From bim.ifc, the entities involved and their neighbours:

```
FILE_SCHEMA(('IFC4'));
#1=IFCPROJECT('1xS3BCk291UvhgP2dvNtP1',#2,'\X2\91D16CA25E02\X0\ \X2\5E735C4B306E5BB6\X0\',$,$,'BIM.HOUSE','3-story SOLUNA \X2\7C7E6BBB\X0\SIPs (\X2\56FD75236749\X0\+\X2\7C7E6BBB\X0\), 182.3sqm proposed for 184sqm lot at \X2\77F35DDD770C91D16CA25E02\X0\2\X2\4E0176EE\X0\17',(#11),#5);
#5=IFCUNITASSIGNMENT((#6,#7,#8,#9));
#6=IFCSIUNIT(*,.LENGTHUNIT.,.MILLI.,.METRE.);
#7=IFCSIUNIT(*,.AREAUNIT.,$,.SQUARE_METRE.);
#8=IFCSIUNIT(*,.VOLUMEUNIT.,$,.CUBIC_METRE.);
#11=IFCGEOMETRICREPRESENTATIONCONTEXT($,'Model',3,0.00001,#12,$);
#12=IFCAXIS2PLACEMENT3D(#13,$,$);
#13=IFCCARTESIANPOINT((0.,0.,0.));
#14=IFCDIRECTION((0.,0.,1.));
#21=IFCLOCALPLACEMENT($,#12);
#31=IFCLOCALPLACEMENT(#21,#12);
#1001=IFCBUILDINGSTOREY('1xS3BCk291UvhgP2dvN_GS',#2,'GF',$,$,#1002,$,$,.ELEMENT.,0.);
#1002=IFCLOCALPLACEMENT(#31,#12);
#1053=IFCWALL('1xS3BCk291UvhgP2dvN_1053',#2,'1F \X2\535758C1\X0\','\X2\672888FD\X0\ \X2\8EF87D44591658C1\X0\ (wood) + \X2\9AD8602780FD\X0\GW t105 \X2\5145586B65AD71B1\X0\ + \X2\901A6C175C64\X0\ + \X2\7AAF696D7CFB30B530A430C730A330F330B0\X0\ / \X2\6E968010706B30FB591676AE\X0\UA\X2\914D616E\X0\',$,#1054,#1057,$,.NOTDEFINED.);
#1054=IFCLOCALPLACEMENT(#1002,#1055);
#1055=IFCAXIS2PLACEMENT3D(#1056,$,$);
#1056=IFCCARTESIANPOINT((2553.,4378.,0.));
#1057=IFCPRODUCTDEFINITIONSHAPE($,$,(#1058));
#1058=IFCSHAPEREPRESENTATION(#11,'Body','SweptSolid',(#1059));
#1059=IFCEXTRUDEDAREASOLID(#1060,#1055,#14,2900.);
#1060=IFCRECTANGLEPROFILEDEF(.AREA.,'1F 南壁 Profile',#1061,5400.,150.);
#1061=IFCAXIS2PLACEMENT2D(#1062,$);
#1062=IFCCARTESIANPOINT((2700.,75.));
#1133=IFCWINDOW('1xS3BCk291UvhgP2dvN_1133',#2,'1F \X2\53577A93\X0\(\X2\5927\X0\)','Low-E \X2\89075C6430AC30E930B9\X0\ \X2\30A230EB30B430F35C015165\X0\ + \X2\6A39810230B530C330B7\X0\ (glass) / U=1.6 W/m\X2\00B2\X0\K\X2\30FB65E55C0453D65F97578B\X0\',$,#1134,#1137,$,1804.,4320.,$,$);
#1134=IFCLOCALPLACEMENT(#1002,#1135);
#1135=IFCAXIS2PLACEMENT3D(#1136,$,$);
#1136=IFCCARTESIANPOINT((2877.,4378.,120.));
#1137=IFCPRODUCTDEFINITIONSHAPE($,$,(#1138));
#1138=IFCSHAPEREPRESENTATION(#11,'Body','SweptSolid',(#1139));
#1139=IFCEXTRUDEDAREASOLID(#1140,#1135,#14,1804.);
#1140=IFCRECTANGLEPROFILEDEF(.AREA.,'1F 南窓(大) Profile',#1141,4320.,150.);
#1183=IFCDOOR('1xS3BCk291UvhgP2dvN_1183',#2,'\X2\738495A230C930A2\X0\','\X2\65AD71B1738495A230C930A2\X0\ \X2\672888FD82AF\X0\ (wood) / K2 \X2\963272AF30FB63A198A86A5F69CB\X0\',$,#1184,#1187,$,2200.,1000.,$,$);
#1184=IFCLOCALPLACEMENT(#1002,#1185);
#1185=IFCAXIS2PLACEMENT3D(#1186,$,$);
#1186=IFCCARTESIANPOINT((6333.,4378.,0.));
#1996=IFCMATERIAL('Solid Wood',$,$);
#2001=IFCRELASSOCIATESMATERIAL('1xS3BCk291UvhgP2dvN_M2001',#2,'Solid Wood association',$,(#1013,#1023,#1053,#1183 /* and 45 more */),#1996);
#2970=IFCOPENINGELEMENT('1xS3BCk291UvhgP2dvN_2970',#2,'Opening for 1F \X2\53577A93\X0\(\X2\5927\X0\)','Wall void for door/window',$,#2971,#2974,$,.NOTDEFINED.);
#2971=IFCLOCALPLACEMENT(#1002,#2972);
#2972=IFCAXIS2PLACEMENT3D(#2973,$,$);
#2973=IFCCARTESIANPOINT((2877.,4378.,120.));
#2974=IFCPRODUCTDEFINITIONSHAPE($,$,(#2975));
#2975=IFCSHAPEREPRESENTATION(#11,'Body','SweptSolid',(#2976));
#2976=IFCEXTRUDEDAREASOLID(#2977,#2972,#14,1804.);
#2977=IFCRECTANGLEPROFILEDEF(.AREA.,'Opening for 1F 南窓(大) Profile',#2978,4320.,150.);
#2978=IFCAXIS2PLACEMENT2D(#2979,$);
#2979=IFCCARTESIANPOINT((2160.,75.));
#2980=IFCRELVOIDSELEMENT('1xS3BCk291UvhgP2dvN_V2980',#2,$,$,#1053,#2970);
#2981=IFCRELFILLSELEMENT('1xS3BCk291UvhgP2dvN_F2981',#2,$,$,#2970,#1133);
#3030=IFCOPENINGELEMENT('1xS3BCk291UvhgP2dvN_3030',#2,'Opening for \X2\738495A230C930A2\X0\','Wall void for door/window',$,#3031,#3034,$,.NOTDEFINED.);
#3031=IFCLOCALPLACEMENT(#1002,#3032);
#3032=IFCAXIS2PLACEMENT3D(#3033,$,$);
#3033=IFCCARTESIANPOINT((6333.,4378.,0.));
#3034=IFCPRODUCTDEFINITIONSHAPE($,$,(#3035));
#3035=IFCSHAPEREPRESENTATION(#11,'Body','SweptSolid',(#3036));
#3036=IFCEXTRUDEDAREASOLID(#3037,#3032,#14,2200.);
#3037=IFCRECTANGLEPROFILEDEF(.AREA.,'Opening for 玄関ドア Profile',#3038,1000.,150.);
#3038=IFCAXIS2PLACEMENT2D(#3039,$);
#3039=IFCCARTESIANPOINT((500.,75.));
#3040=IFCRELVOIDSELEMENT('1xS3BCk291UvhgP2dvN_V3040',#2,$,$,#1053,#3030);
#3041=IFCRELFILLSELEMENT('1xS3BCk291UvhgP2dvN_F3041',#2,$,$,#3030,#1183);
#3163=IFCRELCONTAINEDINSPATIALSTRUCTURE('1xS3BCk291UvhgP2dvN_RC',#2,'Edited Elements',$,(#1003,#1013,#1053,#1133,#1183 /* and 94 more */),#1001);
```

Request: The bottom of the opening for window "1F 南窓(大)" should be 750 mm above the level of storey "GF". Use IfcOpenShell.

```python
import numpy as np
import ifcopenshell
import ifcopenshell.api.geometry
import ifcopenshell.geom
import ifcopenshell.util.element
import ifcopenshell.util.placement
import ifcopenshell.util.shape
import ifcopenshell.util.unit

model = ifcopenshell.open("bim.ifc")
unit_scale = ifcopenshell.util.unit.calculate_unit_scale(model)

window = model.by_guid("1xS3BCk291UvhgP2dvN_1133")
opening = window.FillsVoids[0].RelatingOpeningElement
storey = ifcopenshell.util.element.get_container(window, ifc_class="IfcBuildingStorey")
level = ifcopenshell.util.placement.get_local_placement(storey.ObjectPlacement)[2, 3]

# The opening's origin need not be at the sill, so measure its lowest point.
shape = ifcopenshell.geom.create_shape(ifcopenshell.geom.settings(), opening)
bottom = ifcopenshell.util.shape.get_shape_bottom_elevation(shape, shape.geometry) / unit_scale
dz = level + 750.0 - bottom

shift = np.array([0.0, 0.0, dz])
# The window is not placed relative to its opening, so move both.
for product in (opening, window):
    matrix = ifcopenshell.util.placement.get_local_placement(product.ObjectPlacement)
    matrix[:3, 3] += shift
    ifcopenshell.api.geometry.edit_object_placement(model, product=product, matrix=matrix, is_si=False)

print(f"moved by {dz * unit_scale:+.3f} m")

model.write("bim-out.ifc")
```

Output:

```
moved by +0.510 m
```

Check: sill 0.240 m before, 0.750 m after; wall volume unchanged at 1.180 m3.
